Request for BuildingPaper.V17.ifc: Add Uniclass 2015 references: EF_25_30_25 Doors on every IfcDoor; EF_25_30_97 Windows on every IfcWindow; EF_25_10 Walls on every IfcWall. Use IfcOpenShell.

First a look at what the model holds.

```python
import ifcopenshell

model = ifcopenshell.open("BuildingPaper.V17.ifc")
print(model.schema)
print("classifications:", [c.Name for c in model.by_type("IfcClassification")])
for ifc_class in ("IfcDoor", "IfcRoof", "IfcStair", "IfcWall", "IfcWindow"):
    print(ifc_class, len(model.by_type(ifc_class)))
```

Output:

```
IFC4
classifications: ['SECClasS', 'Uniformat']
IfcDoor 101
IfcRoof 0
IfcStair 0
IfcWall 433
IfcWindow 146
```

```python
import ifcopenshell
import ifcopenshell.api.classification

model = ifcopenshell.open("BuildingPaper.V17.ifc")

system = ifcopenshell.api.classification.add_classification(model, classification="Uniclass 2015")

codes = {
    "IfcDoor": ("EF_25_30_25", "Doors"),
    "IfcWindow": ("EF_25_30_97", "Windows"),
    "IfcWall": ("EF_25_10", "Walls"),
}
for ifc_class, (code, name) in codes.items():
    products = model.by_type(ifc_class)
    ifcopenshell.api.classification.add_reference(
        model, products=products, classification=system, identification=code, name=name
    )
    print(code, len(products))

model.write("BuildingPaper.V17_updated.ifc")
```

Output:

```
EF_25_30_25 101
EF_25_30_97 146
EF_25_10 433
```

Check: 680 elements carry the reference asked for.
